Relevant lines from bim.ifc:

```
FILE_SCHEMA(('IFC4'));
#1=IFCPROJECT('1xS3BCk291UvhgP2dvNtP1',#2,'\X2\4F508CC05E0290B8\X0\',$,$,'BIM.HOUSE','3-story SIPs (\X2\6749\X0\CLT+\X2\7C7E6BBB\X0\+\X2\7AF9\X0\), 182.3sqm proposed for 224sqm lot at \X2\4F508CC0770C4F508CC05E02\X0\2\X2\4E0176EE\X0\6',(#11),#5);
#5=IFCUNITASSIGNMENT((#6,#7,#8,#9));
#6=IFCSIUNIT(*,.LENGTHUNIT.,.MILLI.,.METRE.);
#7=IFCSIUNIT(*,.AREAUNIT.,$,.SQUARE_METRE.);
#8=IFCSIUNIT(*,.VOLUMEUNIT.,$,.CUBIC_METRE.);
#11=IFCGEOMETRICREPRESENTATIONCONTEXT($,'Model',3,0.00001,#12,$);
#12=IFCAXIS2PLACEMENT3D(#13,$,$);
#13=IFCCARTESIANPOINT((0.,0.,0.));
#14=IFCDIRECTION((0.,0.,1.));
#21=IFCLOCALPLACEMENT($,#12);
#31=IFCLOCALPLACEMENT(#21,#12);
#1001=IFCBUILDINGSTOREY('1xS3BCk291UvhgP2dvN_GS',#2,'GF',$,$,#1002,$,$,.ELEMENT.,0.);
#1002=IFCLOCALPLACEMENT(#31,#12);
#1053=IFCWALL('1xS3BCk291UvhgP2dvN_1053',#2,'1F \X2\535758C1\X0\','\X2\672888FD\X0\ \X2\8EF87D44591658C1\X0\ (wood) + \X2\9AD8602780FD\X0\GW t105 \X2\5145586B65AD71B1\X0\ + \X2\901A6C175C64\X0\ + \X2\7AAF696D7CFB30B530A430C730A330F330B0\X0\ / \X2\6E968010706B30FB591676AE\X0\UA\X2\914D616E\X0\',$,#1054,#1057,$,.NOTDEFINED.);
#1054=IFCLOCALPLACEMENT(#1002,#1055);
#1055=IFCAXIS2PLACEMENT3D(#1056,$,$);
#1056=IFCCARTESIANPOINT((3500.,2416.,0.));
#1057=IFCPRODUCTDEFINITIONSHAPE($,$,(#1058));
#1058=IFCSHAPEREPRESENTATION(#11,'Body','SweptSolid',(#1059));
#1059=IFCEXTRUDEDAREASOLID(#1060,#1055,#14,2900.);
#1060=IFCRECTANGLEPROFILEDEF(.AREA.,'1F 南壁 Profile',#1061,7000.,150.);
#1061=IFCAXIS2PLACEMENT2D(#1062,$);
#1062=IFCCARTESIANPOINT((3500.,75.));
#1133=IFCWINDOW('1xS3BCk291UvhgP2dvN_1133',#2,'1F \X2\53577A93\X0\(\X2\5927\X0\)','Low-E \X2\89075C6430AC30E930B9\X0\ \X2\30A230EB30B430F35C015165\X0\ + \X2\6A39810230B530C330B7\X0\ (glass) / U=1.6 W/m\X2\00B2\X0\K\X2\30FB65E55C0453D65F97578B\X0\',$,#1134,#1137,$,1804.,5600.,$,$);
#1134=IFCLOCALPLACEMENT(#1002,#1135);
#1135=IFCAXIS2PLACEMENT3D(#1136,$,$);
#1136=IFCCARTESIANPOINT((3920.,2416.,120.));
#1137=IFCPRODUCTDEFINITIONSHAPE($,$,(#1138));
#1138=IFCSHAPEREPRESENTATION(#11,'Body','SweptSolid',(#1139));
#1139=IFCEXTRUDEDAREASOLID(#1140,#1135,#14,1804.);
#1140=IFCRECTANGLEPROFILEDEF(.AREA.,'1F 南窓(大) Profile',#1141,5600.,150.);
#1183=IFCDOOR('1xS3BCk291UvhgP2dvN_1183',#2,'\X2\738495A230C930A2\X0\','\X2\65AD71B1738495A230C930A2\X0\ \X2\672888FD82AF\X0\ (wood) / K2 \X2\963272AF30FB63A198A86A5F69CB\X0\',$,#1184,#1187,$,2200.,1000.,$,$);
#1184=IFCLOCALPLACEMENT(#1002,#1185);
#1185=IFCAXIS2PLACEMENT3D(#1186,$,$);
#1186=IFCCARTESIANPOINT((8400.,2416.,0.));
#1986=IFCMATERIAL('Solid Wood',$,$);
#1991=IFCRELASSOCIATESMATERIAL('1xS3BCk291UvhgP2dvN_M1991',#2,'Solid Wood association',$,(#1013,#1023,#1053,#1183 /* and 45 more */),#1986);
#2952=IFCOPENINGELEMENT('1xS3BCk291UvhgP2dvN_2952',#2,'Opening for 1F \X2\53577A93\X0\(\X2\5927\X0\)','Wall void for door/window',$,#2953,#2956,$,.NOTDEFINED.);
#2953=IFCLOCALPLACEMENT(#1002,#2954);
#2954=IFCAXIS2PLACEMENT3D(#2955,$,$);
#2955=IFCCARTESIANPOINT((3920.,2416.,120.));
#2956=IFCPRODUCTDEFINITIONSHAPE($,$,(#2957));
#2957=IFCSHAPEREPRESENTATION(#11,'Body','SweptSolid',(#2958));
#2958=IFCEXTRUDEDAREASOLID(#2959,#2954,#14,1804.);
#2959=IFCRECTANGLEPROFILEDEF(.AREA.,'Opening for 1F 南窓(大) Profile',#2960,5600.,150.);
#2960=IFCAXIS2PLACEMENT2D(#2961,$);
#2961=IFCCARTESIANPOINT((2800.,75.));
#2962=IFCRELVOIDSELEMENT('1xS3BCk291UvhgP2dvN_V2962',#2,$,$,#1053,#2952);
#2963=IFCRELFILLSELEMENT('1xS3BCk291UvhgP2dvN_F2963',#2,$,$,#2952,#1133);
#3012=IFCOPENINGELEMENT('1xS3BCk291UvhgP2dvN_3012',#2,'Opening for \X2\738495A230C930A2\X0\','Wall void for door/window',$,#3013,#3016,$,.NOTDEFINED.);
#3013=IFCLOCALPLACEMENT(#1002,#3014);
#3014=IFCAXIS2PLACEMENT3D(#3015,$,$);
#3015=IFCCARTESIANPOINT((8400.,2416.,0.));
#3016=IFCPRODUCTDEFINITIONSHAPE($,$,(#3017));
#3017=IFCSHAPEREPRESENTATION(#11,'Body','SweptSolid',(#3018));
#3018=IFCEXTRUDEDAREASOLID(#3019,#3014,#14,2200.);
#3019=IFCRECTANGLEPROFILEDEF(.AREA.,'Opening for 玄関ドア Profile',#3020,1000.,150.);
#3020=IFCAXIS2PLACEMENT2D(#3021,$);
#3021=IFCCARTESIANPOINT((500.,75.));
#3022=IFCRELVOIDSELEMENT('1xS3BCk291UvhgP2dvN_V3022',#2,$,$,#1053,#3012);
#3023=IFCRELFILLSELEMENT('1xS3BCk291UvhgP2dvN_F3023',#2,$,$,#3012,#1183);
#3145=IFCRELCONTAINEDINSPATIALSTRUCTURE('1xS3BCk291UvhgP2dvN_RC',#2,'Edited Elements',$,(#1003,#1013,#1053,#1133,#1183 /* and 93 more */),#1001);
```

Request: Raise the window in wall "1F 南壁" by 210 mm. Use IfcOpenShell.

```python
import numpy as np
import ifcopenshell
import ifcopenshell.api.geometry
import ifcopenshell.util.placement
import ifcopenshell.util.unit

model = ifcopenshell.open("bim.ifc")
unit_scale = ifcopenshell.util.unit.calculate_unit_scale(model)

window = model.by_guid("1xS3BCk291UvhgP2dvN_1133")
opening = window.FillsVoids[0].RelatingOpeningElement
dz = 0.21 / unit_scale

shift = np.array([0.0, 0.0, dz])
# The window is not placed relative to its opening, so move both.
for product in (opening, window):
    matrix = ifcopenshell.util.placement.get_local_placement(product.ObjectPlacement)
    matrix[:3, 3] += shift
    ifcopenshell.api.geometry.edit_object_placement(model, product=product, matrix=matrix, is_si=False)

print(f"moved by {dz * unit_scale:+.3f} m")

model.write("bim_edited.ifc")
```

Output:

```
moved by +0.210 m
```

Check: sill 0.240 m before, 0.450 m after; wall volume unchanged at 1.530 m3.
